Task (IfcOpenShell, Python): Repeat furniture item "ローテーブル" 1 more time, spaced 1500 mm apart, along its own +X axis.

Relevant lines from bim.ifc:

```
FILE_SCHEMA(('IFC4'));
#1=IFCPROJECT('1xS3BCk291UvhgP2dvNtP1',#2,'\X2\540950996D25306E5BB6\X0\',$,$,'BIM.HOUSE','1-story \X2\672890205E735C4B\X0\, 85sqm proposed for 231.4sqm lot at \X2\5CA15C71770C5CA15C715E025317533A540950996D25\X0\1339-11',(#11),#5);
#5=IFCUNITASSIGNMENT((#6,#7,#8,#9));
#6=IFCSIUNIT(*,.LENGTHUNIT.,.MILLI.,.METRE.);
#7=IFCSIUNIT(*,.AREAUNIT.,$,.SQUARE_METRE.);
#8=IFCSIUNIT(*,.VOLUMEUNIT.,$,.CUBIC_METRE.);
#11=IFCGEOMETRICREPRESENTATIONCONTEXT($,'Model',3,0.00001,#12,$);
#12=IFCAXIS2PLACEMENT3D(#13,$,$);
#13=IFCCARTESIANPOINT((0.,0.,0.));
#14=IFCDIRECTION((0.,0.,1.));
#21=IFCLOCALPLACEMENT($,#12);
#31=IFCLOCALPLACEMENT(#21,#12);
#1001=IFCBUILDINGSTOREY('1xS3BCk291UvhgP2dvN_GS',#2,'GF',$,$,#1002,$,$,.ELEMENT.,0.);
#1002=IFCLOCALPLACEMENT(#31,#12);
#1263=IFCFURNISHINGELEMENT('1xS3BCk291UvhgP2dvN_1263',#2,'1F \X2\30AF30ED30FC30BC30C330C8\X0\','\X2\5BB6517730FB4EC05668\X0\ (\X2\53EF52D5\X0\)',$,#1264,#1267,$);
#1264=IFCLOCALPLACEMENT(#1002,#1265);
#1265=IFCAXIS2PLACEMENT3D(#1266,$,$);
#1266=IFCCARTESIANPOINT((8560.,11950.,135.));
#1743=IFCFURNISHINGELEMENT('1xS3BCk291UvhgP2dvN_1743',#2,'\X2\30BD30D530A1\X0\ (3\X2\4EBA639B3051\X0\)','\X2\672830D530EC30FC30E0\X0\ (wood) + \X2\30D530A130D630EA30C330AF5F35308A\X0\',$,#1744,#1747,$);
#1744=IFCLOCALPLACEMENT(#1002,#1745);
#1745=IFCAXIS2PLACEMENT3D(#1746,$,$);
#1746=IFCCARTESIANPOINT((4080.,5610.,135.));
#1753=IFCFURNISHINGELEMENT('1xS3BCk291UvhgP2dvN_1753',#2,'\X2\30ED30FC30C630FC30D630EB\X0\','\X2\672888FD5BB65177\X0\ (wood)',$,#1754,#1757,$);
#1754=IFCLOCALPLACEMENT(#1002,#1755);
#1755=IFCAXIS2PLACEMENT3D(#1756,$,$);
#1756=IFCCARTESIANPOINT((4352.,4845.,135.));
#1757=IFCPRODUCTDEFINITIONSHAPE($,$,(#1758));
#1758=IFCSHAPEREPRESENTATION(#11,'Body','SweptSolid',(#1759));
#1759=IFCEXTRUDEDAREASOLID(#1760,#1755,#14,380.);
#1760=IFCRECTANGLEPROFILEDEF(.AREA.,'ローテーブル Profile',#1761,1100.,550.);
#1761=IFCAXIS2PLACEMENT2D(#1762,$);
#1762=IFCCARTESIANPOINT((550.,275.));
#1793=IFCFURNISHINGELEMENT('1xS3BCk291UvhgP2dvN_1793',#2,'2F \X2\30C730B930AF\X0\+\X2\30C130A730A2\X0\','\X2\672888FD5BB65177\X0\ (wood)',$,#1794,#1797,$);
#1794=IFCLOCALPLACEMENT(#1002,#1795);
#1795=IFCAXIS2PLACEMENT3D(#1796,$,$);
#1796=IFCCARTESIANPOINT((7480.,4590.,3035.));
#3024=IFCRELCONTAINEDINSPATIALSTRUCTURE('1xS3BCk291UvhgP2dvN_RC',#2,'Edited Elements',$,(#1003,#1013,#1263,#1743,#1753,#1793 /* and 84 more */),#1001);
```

```python
import ifcopenshell
import ifcopenshell.api.geometry
import ifcopenshell.api.root
import ifcopenshell.util.element
import ifcopenshell.util.placement

model = ifcopenshell.open("bim.ifc")


def reuse_history(source, copy):
    """copy_class also copies each property set's owner history, people and application; keep the originals."""
    for rel in copy.IsDefinedBy:
        if rel.is_a("IfcRelDefinesByProperties") and (history := rel.RelatingPropertyDefinition.OwnerHistory):
            rel.RelatingPropertyDefinition.OwnerHistory = source.OwnerHistory
            ifcopenshell.util.element.remove_deep2(model, history)


source = model.by_id(1753)
base = ifcopenshell.util.placement.get_local_placement(source.ObjectPlacement)
step = base[:3, 0] * 1500.0

for i in range(1, 2):
    copy = ifcopenshell.api.root.copy_class(model, product=source)
    copy.Representation = ifcopenshell.util.element.copy_deep(
        model, source.Representation, exclude=["IfcGeometricRepresentationContext", "IfcRepresentationMap"]
    )
    reuse_history(source, copy)
    matrix = base.copy()
    matrix[:3, 3] += i * step
    print("added at", matrix[:3, 3].round(3) + 0.0)
    ifcopenshell.api.geometry.edit_object_placement(model, product=copy, matrix=matrix, is_si=False)

model.write("bim_updated.ifc")
```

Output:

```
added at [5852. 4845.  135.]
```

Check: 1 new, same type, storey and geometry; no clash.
